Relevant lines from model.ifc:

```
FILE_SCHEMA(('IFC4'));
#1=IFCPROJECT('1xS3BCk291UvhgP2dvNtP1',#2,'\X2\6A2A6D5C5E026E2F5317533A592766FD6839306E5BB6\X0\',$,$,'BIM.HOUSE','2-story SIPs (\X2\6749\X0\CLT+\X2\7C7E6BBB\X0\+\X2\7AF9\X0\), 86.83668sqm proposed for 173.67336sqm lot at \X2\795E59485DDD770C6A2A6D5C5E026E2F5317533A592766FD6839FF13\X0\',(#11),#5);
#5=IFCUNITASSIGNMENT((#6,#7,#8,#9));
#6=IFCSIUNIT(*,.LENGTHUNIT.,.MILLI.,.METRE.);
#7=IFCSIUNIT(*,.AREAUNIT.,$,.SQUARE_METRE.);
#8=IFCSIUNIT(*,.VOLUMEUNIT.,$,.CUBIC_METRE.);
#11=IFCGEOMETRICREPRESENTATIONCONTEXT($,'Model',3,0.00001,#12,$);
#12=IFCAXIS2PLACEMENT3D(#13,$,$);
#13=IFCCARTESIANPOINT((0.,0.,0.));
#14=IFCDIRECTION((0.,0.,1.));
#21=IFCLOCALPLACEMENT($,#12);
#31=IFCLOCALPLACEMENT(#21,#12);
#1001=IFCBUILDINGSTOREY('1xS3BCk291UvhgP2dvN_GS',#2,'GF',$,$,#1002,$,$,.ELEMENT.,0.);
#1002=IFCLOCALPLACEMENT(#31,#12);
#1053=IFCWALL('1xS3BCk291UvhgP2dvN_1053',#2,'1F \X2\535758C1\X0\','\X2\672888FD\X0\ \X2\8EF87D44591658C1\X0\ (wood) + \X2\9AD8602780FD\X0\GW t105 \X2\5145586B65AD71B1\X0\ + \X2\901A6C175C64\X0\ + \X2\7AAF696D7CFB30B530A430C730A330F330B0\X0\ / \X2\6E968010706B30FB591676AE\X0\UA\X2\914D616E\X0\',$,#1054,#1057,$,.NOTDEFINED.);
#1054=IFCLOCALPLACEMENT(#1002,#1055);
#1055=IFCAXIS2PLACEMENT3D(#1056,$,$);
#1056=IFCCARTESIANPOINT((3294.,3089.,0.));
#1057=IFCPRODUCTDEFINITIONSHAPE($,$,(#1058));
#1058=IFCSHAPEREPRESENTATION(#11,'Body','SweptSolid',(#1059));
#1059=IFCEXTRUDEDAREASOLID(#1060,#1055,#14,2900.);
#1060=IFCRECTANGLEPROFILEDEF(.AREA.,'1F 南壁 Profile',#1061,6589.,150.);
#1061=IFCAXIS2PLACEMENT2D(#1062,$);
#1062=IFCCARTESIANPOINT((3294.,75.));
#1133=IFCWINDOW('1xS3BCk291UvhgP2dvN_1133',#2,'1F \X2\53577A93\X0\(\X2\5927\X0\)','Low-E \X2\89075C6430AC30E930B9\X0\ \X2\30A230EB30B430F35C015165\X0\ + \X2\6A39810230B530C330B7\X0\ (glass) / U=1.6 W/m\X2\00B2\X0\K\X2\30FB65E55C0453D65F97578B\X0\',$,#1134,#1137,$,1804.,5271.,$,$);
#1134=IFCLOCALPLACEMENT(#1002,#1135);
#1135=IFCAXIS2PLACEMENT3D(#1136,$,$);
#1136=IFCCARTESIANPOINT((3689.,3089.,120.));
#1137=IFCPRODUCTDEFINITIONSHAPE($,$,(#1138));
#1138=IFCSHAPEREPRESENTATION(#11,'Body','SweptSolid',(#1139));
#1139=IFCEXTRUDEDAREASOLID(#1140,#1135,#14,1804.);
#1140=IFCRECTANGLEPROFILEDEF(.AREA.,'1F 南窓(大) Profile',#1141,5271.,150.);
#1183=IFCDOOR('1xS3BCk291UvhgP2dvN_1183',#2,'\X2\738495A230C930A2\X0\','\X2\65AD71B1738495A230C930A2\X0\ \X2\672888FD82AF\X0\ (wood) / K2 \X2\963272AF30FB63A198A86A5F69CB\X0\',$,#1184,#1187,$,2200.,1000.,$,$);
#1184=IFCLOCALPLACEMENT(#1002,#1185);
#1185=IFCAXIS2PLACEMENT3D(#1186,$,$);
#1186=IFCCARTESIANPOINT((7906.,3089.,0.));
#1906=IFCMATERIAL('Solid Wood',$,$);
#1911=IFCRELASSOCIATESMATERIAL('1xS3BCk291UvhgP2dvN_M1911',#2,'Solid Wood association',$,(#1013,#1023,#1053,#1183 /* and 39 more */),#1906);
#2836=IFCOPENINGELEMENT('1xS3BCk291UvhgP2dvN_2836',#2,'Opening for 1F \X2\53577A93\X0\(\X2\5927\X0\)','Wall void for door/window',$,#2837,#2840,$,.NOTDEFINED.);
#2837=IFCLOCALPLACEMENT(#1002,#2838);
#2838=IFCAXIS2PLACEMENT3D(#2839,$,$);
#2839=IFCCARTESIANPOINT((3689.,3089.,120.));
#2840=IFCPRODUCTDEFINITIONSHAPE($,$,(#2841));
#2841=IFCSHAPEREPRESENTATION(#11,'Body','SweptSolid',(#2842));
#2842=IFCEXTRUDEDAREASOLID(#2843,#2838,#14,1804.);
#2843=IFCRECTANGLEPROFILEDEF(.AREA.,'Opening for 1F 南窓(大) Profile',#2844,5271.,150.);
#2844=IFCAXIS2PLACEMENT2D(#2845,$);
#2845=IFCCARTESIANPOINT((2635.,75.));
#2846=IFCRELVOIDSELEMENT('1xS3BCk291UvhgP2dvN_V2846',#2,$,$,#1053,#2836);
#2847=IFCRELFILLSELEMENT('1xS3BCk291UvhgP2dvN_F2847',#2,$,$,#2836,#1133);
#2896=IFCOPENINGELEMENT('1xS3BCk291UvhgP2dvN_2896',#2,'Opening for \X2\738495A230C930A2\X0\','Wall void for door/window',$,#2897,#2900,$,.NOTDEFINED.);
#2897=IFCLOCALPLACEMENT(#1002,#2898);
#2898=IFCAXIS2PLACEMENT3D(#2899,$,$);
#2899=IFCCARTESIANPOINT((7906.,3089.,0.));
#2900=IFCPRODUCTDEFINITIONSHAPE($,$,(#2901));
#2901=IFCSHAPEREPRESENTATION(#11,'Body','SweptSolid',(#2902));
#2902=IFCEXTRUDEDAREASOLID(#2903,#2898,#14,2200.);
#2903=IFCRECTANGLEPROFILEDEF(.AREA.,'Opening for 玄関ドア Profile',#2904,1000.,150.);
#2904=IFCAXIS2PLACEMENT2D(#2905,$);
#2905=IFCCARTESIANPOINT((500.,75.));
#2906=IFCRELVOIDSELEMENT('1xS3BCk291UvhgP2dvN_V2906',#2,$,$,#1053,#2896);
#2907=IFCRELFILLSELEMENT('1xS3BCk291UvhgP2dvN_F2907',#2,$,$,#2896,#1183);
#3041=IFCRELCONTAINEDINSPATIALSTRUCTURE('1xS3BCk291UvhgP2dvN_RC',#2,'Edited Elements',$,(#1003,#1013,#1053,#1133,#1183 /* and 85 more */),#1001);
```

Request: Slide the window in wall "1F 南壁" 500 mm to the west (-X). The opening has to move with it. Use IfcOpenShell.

```python
import ifcopenshell
import ifcopenshell.api.geometry
import ifcopenshell.util.placement

model = ifcopenshell.open("model.ifc")

window = model.by_guid("1xS3BCk291UvhgP2dvN_1133")
opening = window.FillsVoids[0].RelatingOpeningElement
wall = opening.VoidsElements[0].RelatingBuildingElement

wall_matrix = ifcopenshell.util.placement.get_local_placement(wall.ObjectPlacement)
shift = wall_matrix[:3, 0] * -500.0
before = ifcopenshell.util.placement.get_local_placement(window.ObjectPlacement)[:3, 3].copy()

# The window is not placed relative to its opening, so move both.
for product in (opening, window):
    matrix = ifcopenshell.util.placement.get_local_placement(product.ObjectPlacement)
    matrix[:3, 3] += shift
    ifcopenshell.api.geometry.edit_object_placement(model, product=product, matrix=matrix, is_si=False)

after = ifcopenshell.util.placement.get_local_placement(window.ObjectPlacement)[:3, 3]
print("window moved by", (after - before).round(3) + 0.0)

model.write("model_updated.ifc")
```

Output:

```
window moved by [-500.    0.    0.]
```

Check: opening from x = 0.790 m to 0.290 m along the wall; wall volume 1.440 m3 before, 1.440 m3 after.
